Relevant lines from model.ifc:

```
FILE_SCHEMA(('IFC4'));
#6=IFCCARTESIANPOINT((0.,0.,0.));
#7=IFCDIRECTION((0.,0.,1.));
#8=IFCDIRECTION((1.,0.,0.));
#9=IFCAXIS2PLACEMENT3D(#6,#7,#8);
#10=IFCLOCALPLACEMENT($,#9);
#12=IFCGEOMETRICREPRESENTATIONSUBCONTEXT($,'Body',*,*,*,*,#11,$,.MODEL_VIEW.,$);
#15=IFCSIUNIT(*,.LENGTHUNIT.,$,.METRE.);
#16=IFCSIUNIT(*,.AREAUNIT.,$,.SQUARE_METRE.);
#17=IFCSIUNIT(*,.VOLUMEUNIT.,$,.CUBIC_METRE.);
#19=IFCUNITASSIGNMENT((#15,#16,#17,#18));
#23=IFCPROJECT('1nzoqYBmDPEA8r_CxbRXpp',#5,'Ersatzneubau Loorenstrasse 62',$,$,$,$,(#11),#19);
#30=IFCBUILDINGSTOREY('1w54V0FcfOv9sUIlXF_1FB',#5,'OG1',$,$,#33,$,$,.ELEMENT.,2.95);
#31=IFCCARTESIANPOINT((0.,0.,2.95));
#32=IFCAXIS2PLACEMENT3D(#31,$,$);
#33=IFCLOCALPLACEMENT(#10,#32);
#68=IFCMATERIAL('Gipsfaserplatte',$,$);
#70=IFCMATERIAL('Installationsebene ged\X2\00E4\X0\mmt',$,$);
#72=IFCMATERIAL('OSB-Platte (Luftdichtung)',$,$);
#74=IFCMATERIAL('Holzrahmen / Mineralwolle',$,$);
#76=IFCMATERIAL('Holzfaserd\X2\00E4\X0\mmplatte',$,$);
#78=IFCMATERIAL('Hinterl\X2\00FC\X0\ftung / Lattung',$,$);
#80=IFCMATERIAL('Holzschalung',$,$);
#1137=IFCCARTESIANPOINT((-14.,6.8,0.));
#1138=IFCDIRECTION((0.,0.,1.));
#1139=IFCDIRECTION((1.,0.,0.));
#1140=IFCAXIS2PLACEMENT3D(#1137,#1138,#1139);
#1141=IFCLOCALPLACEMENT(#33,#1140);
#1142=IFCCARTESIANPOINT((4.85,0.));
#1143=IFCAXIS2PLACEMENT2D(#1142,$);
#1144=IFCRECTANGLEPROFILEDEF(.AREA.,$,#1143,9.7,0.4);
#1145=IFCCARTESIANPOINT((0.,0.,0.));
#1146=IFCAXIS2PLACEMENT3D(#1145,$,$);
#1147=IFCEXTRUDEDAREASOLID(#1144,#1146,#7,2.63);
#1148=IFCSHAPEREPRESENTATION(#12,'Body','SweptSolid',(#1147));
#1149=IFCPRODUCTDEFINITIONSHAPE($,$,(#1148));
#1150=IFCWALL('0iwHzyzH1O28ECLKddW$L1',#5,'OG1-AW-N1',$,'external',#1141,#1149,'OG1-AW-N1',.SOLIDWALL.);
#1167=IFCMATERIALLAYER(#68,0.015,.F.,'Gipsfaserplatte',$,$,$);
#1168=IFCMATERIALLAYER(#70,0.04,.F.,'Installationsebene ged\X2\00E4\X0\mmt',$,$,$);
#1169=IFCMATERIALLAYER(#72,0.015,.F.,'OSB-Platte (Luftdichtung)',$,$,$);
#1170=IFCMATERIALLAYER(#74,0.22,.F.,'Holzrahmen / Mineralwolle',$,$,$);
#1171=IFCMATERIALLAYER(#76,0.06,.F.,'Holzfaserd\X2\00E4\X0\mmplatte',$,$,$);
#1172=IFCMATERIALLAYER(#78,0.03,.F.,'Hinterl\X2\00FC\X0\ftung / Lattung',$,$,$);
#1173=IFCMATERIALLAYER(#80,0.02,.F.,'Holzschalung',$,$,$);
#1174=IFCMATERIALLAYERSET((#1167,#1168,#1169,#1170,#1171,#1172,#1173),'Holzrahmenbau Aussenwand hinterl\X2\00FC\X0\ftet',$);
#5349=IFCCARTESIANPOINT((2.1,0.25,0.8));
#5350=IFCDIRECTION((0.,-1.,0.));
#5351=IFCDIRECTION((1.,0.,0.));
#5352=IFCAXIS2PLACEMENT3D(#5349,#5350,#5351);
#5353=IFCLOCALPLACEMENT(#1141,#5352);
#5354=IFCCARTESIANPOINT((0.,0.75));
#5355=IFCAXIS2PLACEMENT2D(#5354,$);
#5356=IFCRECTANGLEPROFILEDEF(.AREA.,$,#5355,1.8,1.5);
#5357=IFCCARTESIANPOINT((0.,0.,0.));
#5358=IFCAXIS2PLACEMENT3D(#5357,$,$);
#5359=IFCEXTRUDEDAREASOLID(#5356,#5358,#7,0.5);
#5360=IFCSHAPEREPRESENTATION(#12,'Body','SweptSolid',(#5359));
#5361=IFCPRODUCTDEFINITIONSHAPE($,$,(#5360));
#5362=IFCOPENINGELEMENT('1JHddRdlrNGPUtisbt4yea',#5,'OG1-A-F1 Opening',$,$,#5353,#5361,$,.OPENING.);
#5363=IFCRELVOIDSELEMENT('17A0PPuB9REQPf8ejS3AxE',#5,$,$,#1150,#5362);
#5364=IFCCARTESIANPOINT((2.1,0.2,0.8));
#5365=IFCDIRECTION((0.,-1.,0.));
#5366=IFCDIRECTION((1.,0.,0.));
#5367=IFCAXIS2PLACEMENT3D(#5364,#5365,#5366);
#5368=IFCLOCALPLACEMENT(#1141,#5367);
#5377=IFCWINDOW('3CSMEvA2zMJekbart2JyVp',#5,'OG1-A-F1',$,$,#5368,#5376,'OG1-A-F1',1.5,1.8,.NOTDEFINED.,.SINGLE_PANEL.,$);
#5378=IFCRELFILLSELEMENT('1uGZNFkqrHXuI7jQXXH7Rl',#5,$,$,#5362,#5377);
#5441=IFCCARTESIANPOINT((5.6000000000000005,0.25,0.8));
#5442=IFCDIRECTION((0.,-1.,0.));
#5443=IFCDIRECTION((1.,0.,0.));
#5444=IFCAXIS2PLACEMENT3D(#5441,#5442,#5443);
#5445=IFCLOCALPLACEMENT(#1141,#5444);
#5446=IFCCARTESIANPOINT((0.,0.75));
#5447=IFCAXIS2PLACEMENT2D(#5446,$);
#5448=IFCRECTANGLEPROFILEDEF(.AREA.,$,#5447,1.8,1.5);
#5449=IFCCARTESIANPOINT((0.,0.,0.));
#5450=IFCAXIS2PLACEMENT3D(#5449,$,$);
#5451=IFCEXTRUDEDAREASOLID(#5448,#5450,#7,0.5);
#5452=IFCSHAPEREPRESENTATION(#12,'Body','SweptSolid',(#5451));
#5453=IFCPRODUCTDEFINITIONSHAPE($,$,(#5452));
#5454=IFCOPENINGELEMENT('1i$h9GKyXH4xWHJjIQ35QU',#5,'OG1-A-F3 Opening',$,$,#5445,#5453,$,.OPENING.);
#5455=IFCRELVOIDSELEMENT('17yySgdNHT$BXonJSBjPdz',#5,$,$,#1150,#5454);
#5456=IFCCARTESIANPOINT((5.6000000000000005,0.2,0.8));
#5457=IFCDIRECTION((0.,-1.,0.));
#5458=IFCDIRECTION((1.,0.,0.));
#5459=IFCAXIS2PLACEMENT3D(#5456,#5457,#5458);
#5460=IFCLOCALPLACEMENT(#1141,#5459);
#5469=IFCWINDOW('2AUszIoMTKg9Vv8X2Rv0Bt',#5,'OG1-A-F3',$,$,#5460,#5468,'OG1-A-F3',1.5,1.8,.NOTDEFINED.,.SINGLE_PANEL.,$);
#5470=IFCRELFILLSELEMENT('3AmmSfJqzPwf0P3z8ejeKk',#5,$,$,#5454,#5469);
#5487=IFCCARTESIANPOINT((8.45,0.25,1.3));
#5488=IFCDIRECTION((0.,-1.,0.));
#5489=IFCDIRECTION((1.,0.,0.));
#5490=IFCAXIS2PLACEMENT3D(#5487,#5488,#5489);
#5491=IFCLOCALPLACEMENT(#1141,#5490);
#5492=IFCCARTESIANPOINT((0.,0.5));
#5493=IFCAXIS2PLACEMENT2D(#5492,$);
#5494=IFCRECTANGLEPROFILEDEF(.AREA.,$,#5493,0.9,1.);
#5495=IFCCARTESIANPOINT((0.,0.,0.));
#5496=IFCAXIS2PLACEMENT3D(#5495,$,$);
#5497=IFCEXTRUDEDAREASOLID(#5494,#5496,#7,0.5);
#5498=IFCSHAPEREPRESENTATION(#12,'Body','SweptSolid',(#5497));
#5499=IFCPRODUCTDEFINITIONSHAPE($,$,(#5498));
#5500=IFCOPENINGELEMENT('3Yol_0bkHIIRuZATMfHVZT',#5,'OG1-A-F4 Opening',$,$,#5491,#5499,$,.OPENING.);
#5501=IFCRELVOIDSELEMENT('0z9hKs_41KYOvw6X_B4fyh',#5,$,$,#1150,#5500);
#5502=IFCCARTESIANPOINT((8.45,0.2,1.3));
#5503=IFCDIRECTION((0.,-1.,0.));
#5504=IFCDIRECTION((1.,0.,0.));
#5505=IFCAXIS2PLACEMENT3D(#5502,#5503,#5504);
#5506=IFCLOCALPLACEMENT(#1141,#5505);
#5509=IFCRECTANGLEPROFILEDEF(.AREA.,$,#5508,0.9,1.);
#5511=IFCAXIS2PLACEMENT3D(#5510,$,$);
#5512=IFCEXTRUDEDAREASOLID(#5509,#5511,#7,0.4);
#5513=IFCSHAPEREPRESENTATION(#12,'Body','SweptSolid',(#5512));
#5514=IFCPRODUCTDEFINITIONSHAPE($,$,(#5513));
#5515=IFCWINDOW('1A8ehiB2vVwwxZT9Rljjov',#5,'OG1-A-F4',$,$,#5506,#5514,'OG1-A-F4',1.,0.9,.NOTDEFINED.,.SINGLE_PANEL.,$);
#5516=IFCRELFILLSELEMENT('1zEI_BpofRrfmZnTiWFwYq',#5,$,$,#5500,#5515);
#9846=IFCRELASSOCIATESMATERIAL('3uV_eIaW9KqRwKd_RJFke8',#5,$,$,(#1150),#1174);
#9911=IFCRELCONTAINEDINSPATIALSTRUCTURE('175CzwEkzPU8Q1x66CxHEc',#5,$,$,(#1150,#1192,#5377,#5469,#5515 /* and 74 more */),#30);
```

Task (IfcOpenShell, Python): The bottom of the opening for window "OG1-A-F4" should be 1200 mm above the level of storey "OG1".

```python
import numpy as np
import ifcopenshell
import ifcopenshell.api.geometry
import ifcopenshell.geom
import ifcopenshell.util.element
import ifcopenshell.util.placement
import ifcopenshell.util.shape
import ifcopenshell.util.unit

model = ifcopenshell.open("model.ifc")
unit_scale = ifcopenshell.util.unit.calculate_unit_scale(model)

window = model.by_guid("1A8ehiB2vVwwxZT9Rljjov")
opening = window.FillsVoids[0].RelatingOpeningElement
storey = ifcopenshell.util.element.get_container(window, ifc_class="IfcBuildingStorey")
level = ifcopenshell.util.placement.get_local_placement(storey.ObjectPlacement)[2, 3]

# The opening's origin need not be at the sill, so measure its lowest point.
shape = ifcopenshell.geom.create_shape(ifcopenshell.geom.settings(), opening)
bottom = ifcopenshell.util.shape.get_shape_bottom_elevation(shape, shape.geometry) / unit_scale
dz = level + 1.2 - bottom

shift = np.array([0.0, 0.0, dz])
# The window is not placed relative to its opening, so move both.
for product in (opening, window):
    matrix = ifcopenshell.util.placement.get_local_placement(product.ObjectPlacement)
    matrix[:3, 3] += shift
    ifcopenshell.api.geometry.edit_object_placement(model, product=product, matrix=matrix, is_si=False)

print(f"moved by {dz * unit_scale:+.3f} m")

model.write("model_v2.ifc")
```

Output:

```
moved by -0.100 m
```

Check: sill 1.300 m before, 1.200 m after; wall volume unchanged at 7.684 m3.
